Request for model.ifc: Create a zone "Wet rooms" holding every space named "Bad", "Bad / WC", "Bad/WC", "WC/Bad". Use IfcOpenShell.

First a look at what the model holds.

```python
import ifcopenshell

model = ifcopenshell.open("model.ifc")
print(model.schema)
seen = {}
for space in model.by_type("IfcSpace"):
    seen[space.LongName] = seen.get(space.LongName, 0) + 1
for name, count in sorted(seen.items(), key=str):
    print(count, "x", name)
print("zones:", [z.Name for z in model.by_type("IfcZone")][:20])
```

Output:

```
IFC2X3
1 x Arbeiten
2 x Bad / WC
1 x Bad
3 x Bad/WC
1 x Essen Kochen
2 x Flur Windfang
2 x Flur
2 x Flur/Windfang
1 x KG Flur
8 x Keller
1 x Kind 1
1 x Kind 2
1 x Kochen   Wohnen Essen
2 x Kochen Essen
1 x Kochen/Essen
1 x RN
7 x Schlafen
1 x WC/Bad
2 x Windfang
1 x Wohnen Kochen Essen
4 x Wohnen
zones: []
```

```python
import ifcopenshell
import ifcopenshell.api.group
import ifcopenshell.api.root

model = ifcopenshell.open("model.ifc")

names = {"Bad", "Bad / WC", "Bad/WC", "WC/Bad"}
spaces = [s for s in model.by_type("IfcSpace") if s.LongName in names]

zone = ifcopenshell.api.root.create_entity(model, ifc_class="IfcZone", name="Wet rooms")
ifcopenshell.api.group.assign_group(model, products=spaces, group=zone)
print(len(spaces), "spaces in", zone.Name)

model.write("model_edited.ifc")
```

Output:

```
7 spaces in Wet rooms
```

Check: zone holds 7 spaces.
